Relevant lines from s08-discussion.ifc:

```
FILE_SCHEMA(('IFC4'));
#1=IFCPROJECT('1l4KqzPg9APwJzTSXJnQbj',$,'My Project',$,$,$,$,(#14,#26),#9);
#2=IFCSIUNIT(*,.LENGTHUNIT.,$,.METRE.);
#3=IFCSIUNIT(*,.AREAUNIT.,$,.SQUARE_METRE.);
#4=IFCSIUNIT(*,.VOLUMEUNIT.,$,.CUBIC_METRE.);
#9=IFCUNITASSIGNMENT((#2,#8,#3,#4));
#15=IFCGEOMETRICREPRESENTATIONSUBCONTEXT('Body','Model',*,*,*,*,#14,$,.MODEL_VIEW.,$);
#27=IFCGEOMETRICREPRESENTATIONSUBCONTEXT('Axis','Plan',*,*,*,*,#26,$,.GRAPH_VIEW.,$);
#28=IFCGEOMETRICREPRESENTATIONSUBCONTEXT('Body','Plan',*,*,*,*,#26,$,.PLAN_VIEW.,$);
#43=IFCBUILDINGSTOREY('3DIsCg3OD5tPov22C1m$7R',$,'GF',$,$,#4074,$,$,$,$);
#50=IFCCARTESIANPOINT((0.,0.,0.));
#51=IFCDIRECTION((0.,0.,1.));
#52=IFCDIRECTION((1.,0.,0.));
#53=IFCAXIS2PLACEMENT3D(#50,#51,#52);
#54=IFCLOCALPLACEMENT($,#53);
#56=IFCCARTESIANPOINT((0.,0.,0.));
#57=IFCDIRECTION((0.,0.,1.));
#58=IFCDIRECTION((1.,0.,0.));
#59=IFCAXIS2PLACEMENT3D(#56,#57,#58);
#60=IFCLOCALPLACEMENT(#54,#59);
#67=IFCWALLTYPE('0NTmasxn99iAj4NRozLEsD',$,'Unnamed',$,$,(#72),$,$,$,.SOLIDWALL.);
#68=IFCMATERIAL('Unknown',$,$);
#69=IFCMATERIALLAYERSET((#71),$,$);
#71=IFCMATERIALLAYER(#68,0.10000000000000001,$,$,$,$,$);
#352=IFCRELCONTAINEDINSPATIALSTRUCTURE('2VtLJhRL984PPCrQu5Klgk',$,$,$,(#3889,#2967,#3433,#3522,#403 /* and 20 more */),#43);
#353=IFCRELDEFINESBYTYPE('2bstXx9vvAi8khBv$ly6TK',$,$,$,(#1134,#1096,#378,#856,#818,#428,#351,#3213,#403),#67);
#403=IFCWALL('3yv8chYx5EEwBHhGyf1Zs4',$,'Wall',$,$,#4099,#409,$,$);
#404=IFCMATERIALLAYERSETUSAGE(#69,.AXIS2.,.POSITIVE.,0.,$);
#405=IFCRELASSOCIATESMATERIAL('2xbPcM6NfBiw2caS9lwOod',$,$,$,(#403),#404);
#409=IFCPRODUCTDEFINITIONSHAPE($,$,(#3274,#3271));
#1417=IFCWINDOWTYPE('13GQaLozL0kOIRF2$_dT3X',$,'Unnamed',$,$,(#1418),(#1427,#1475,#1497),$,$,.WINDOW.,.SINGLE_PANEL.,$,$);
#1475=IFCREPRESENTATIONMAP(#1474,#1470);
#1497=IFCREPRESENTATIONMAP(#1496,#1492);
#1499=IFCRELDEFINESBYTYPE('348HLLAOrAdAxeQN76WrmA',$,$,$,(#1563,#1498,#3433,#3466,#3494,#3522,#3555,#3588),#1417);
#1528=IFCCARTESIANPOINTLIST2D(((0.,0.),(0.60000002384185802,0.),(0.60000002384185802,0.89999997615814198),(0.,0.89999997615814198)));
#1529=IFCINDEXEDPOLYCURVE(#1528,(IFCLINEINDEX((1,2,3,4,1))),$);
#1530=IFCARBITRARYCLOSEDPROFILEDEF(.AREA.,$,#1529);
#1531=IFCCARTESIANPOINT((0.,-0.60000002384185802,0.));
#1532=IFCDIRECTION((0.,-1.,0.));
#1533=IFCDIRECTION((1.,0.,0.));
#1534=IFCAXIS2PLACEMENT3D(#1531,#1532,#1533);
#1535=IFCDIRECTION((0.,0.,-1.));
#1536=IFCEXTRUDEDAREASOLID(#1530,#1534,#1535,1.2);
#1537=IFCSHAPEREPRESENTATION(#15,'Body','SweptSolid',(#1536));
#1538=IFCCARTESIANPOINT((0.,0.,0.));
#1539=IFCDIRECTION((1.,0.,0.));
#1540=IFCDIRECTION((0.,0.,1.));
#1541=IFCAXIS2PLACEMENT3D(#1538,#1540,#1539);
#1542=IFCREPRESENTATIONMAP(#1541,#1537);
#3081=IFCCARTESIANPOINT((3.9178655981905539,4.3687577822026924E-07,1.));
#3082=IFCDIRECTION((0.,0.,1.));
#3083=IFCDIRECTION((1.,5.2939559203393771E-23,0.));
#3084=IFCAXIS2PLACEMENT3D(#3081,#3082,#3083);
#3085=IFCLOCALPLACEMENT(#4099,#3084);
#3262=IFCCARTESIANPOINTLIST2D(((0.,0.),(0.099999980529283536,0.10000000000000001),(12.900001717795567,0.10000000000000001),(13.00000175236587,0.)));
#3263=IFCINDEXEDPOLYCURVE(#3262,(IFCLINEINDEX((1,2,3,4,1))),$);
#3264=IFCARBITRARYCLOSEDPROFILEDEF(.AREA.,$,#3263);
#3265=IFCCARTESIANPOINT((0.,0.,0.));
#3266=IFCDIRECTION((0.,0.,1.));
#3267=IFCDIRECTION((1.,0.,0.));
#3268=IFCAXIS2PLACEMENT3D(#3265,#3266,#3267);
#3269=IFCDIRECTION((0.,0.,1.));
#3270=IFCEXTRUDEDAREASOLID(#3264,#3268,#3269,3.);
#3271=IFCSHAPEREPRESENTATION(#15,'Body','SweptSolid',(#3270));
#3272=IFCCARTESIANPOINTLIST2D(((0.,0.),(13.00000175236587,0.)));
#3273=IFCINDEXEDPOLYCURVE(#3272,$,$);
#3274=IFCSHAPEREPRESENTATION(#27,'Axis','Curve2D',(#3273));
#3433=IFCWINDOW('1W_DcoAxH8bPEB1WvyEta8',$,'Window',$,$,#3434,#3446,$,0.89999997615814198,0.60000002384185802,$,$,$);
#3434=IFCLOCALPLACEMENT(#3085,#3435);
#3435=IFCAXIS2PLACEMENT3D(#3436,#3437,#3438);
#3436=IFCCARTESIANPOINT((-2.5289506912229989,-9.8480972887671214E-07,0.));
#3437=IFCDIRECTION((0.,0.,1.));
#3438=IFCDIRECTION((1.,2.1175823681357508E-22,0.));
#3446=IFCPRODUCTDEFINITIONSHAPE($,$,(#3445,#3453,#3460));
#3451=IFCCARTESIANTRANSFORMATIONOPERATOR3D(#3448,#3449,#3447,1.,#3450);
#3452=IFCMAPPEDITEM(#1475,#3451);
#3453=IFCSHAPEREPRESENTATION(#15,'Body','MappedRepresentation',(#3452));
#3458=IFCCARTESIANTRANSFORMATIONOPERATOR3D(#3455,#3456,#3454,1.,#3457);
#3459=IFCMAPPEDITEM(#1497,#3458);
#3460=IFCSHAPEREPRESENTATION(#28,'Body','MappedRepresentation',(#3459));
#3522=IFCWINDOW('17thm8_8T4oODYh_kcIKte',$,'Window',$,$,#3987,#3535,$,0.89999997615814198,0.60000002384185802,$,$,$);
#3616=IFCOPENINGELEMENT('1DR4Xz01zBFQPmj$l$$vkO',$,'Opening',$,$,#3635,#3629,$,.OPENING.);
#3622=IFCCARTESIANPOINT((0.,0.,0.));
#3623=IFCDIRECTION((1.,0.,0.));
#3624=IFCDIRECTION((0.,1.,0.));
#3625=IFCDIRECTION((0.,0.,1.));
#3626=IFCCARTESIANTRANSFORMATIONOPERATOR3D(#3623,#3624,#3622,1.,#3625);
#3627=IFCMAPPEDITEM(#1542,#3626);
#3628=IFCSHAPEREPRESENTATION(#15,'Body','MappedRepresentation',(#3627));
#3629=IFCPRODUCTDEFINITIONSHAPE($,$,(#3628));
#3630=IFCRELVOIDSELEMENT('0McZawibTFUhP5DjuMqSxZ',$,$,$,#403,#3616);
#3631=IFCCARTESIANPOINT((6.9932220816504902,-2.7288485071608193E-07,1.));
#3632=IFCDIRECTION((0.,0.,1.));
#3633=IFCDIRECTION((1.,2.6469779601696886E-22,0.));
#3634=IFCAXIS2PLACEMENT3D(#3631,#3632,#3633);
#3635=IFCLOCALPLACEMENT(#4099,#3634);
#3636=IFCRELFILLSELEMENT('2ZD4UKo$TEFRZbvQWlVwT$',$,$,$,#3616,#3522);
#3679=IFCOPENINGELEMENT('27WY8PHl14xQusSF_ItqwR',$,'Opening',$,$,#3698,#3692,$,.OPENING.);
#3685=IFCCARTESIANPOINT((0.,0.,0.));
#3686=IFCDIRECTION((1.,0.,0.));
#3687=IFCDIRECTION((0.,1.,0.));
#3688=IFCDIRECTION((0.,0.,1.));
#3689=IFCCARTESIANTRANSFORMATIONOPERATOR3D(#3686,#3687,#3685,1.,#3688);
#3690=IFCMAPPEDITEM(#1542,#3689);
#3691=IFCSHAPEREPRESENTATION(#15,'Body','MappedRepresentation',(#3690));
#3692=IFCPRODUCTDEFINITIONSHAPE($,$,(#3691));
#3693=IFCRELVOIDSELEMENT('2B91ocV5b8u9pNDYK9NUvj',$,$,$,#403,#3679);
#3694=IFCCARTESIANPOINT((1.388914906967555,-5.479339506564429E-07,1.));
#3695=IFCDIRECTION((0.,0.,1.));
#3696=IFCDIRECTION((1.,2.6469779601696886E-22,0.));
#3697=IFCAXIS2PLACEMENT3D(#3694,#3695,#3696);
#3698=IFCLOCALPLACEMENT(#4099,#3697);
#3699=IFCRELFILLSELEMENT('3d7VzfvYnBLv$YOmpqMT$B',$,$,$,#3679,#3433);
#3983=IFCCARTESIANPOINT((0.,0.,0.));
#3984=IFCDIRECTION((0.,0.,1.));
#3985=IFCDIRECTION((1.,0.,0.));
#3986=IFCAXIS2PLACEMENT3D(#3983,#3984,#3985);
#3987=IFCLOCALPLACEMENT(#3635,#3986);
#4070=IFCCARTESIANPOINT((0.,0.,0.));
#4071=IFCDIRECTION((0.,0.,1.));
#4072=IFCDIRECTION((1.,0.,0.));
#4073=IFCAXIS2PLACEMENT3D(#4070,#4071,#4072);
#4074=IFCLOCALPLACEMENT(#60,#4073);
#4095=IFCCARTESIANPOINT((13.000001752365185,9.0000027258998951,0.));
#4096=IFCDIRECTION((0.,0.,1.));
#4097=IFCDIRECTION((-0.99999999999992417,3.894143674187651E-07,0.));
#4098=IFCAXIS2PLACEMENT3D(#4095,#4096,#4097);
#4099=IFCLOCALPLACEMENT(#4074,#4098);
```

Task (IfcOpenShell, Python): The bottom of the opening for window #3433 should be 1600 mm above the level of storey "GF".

```python
import numpy as np
import ifcopenshell
import ifcopenshell.api.geometry
import ifcopenshell.geom
import ifcopenshell.util.element
import ifcopenshell.util.placement
import ifcopenshell.util.shape
import ifcopenshell.util.unit

model = ifcopenshell.open("s08-discussion.ifc")
unit_scale = ifcopenshell.util.unit.calculate_unit_scale(model)

window = model.by_id(3433)
opening = window.FillsVoids[0].RelatingOpeningElement
storey = ifcopenshell.util.element.get_container(window, ifc_class="IfcBuildingStorey")
level = ifcopenshell.util.placement.get_local_placement(storey.ObjectPlacement)[2, 3]

# The opening's origin need not be at the sill, so measure its lowest point.
shape = ifcopenshell.geom.create_shape(ifcopenshell.geom.settings(), opening)
bottom = ifcopenshell.util.shape.get_shape_bottom_elevation(shape, shape.geometry) / unit_scale
dz = level + 1.6 / unit_scale - bottom

shift = np.array([0.0, 0.0, dz])
# The window is not placed relative to its opening, so move both.
for product in (opening, window):
    matrix = ifcopenshell.util.placement.get_local_placement(product.ObjectPlacement)
    matrix[:3, 3] += shift
    ifcopenshell.api.geometry.edit_object_placement(model, product=product, matrix=matrix, is_si=False)

print(f"moved by {dz * unit_scale:+.3f} m")

model.write("s08-discussion_v2.ifc")
```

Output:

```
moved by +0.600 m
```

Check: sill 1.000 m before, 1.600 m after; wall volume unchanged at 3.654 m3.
